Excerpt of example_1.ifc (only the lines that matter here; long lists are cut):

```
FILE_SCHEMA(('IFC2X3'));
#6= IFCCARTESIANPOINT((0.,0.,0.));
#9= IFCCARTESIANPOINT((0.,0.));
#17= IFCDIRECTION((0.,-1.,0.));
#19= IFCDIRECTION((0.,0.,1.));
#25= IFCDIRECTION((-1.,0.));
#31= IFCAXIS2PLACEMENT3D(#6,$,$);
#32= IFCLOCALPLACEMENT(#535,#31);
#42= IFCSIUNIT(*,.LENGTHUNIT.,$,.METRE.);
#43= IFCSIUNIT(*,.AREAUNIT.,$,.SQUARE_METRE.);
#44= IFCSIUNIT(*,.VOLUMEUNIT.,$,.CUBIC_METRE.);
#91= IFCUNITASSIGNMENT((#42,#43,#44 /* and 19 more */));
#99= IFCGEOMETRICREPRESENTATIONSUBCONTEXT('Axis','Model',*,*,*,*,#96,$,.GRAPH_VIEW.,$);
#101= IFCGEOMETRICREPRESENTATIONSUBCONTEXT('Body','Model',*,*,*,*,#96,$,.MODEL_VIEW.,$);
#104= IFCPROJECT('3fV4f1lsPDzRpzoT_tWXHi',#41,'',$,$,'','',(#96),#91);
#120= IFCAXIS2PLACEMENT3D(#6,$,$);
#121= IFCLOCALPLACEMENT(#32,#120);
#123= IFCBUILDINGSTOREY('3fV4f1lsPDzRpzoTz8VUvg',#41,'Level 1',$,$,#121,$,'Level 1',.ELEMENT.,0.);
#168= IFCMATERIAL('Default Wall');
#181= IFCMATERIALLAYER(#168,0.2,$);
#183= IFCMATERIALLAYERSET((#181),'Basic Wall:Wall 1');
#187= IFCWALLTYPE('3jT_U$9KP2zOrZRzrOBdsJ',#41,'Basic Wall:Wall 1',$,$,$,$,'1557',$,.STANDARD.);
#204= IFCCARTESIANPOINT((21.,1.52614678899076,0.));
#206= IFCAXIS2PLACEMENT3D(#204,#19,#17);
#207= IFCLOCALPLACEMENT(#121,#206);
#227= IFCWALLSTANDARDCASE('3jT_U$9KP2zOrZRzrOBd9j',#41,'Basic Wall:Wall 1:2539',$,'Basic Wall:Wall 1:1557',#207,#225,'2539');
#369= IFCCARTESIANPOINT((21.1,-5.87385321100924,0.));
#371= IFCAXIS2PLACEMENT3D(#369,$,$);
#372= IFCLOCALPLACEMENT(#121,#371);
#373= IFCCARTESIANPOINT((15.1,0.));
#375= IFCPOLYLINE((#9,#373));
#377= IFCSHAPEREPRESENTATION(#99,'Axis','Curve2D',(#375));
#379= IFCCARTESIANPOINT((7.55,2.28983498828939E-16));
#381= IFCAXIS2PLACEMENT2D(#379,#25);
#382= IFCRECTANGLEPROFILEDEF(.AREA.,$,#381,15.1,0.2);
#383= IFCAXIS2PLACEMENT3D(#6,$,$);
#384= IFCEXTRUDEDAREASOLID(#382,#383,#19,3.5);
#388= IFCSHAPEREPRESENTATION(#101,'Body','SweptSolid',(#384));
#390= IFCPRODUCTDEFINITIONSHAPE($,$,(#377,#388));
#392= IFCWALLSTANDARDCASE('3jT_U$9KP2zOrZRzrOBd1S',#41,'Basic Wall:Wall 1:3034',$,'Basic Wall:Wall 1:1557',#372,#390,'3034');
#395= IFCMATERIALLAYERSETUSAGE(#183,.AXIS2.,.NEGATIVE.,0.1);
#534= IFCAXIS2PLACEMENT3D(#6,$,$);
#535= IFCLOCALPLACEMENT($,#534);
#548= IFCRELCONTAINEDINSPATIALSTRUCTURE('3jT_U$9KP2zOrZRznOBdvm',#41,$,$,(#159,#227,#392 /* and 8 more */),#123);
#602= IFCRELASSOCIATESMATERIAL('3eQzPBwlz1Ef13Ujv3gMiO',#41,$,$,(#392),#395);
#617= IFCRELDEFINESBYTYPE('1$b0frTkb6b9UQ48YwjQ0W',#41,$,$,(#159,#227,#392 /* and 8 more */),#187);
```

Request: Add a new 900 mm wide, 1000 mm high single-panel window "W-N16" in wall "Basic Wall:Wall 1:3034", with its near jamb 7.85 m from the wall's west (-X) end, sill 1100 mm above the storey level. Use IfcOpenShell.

```python
import numpy as np
import ifcopenshell
import ifcopenshell.api.feature
import ifcopenshell.api.geometry
import ifcopenshell.api.root
import ifcopenshell.api.spatial
import ifcopenshell.api.type
import ifcopenshell.geom
import ifcopenshell.util.element
import ifcopenshell.util.placement
import ifcopenshell.util.representation
import ifcopenshell.util.shape
import ifcopenshell.util.unit

model = ifcopenshell.open("example_1.ifc")
unit_scale = ifcopenshell.util.unit.calculate_unit_scale(model)
settings = ifcopenshell.geom.settings()


def volume(element):
    """Net volume in cubic metres, openings subtracted."""
    shape = ifcopenshell.geom.create_shape(settings, element)
    return ifcopenshell.util.shape.get_volume(shape.geometry)


wall = model.by_id(392)
storey = ifcopenshell.util.element.get_container(wall, ifc_class="IfcBuildingStorey")
context = ifcopenshell.util.representation.get_context(model, "Model", "Body", "MODEL_VIEW")
before = volume(wall)

width, height, from_end, sill = 0.9, 1, 7.85, 1.1  # metres

# The wall runs along its own X axis, and the end named is its -X end.
wall_shape = ifcopenshell.geom.create_shape(settings, wall)
x, y, z = ifcopenshell.util.shape.get_vertices(wall_shape.geometry).T
start = x.min() + from_end
face, thickness = float(y.min()), float(y.max() - y.min())
wall_matrix = ifcopenshell.util.placement.get_local_placement(wall.ObjectPlacement)
level = ifcopenshell.util.placement.get_local_placement(storey.ObjectPlacement)[2, 3]


def in_wall(x, y):
    """Placement at x, y metres in the wall's axes, at sill height."""
    matrix = wall_matrix.copy()
    matrix[:, 3] = wall_matrix @ np.array([x / unit_scale, y / unit_scale, 0.0, 1.0])
    matrix[2, 3] = level + sill / unit_scale
    return matrix


# Opening: a box that overshoots both wall faces by 50 mm.
opening = ifcopenshell.api.root.create_entity(model, ifc_class="IfcOpeningElement")
box = ifcopenshell.api.geometry.add_wall_representation(
    model, context=context, length=width, height=height, thickness=thickness + 0.1
)
ifcopenshell.api.geometry.assign_representation(model, product=opening, representation=box)
ifcopenshell.api.geometry.edit_object_placement(model, product=opening, matrix=in_wall(start, face - 0.05), is_si=False)
ifcopenshell.api.feature.add_feature(model, feature=opening, element=wall)

window = ifcopenshell.api.root.create_entity(model, ifc_class="IfcWindow", name="W-N16")
window.OverallWidth, window.OverallHeight = width / unit_scale, height / unit_scale
body = ifcopenshell.api.geometry.add_window_representation(
    model,
    context=context,
    overall_width=window.OverallWidth,
    overall_height=window.OverallHeight,
    partition_type="SINGLE_PANEL",
)
ifcopenshell.api.geometry.assign_representation(model, product=window, representation=body)
ifcopenshell.api.spatial.assign_container(model, products=[window], relating_structure=storey)
fills = ifcopenshell.api.feature.add_filling(model, opening=opening, element=window)
fills.OwnerHistory = window.OwnerHistory  # required in IFC2X3

# IFC2X3 keeps the operation on the window style.
style = ifcopenshell.api.root.create_entity(model, ifc_class="IfcWindowStyle", name="W-N16")
style.OperationType, style.ConstructionType = "SINGLE_PANEL", "NOTDEFINED"
style.ParameterTakesPrecedence = style.Sizeable = False
ifcopenshell.api.type.assign_type(model, related_objects=[window], relating_type=style)

# Centre the window in the wall's thickness.
ifcopenshell.api.geometry.edit_object_placement(model, product=window, matrix=in_wall(start, face), is_si=False)
window_shape = ifcopenshell.geom.create_shape(settings, window)
depth = ifcopenshell.util.shape.get_vertices(window_shape.geometry)[:, 1]
offset = face + thickness / 2 - (depth.min() + depth.max()) / 2
ifcopenshell.api.geometry.edit_object_placement(model, product=window, matrix=in_wall(start, offset), is_si=False)

after = volume(wall)

print(f"wall volume {before:.3f} -> {after:.3f} m3")

model.write("example_1_updated.ifc")
```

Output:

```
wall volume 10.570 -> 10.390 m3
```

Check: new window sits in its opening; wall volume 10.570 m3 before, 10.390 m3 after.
